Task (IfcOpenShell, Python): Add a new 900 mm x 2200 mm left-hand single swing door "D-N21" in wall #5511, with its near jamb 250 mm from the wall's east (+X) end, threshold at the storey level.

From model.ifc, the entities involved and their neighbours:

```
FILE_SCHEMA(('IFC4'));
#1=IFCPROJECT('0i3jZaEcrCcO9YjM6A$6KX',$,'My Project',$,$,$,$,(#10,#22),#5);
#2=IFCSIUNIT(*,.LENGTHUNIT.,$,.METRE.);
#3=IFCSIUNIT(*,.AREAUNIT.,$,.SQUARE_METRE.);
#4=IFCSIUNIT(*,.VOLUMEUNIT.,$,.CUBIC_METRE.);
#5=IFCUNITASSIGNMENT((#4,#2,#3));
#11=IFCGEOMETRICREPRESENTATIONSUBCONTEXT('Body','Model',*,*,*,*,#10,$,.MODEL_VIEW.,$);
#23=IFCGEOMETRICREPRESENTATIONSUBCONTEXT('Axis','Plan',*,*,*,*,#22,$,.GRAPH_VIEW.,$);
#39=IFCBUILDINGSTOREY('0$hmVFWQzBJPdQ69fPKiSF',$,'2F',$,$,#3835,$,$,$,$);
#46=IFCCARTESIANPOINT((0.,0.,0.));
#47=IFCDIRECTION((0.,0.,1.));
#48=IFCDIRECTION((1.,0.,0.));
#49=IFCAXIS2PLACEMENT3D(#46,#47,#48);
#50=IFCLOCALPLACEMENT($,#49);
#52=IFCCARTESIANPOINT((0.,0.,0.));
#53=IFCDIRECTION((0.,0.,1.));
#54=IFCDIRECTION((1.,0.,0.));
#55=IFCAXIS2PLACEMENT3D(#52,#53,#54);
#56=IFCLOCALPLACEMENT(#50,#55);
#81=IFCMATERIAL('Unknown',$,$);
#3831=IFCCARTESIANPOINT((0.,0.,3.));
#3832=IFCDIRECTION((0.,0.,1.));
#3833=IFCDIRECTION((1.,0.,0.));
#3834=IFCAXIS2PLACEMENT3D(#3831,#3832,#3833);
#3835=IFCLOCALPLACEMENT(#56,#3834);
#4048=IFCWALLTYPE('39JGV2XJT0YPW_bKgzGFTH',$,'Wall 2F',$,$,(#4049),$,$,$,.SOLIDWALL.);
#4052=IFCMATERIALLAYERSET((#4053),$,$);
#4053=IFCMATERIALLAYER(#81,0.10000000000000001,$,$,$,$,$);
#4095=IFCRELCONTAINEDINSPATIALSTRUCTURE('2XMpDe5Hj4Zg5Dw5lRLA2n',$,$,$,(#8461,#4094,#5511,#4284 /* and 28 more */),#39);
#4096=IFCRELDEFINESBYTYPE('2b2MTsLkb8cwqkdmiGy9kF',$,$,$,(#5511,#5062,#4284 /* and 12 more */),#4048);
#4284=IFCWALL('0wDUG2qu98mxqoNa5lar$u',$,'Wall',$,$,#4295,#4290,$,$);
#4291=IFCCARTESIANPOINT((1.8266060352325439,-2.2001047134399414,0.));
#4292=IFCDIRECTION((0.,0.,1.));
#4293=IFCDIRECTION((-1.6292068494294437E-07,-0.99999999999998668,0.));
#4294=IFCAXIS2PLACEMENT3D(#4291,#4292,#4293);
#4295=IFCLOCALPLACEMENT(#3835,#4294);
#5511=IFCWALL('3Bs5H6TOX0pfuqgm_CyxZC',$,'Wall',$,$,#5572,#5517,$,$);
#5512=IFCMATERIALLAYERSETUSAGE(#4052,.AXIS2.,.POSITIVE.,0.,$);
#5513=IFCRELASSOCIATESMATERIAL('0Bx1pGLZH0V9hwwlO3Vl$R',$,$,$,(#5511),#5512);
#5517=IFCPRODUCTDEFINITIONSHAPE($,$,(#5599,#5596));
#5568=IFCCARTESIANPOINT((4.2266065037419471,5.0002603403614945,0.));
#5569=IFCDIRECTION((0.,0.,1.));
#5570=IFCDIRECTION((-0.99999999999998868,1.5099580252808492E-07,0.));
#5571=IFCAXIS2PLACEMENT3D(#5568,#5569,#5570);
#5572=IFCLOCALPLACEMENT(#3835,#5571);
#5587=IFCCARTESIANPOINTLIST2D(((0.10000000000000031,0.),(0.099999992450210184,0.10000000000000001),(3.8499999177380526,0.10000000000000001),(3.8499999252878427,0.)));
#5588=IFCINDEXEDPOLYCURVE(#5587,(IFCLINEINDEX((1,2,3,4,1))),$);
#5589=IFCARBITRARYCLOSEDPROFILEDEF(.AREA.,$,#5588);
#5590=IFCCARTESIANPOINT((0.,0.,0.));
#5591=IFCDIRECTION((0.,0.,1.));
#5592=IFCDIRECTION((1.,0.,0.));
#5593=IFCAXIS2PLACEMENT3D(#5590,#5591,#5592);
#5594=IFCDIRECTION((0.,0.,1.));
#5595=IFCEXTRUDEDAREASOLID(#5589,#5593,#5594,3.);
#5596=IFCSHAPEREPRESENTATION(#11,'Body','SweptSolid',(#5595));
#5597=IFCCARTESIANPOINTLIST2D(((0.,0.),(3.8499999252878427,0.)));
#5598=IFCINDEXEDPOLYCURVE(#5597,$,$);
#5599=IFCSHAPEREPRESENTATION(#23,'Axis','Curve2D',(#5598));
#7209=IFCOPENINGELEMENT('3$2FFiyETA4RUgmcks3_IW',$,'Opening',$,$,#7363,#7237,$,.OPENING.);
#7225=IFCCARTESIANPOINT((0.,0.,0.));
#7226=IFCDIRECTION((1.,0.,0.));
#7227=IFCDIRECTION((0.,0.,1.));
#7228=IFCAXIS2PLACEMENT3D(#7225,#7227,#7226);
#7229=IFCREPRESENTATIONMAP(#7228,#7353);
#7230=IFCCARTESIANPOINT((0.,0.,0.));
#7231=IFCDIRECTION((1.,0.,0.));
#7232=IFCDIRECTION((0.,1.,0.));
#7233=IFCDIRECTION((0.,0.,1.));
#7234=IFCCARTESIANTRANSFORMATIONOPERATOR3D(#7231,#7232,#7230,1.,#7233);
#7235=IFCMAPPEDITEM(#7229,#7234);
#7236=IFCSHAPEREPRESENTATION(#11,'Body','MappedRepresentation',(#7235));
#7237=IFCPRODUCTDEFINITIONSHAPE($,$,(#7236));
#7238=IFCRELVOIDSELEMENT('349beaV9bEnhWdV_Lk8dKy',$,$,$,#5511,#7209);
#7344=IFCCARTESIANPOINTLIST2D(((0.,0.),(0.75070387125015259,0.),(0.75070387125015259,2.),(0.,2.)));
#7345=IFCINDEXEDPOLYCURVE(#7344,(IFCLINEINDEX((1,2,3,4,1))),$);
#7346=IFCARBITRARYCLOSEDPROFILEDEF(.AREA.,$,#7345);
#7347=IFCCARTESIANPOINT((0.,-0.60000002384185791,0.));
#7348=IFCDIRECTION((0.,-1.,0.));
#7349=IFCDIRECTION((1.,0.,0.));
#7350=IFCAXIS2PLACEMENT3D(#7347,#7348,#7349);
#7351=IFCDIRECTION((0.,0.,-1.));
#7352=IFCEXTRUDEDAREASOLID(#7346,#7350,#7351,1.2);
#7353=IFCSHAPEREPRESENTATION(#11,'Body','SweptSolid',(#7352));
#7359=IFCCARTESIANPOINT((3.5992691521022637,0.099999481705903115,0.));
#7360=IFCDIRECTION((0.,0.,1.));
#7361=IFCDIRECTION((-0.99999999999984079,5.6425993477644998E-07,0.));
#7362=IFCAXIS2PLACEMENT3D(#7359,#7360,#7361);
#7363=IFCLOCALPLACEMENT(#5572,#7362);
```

```python
import numpy as np
import ifcopenshell
import ifcopenshell.api.feature
import ifcopenshell.api.geometry
import ifcopenshell.api.root
import ifcopenshell.api.spatial
import ifcopenshell.geom
import ifcopenshell.util.element
import ifcopenshell.util.placement
import ifcopenshell.util.representation
import ifcopenshell.util.shape
import ifcopenshell.util.unit

model = ifcopenshell.open("model.ifc")
unit_scale = ifcopenshell.util.unit.calculate_unit_scale(model)
settings = ifcopenshell.geom.settings()


def volume(element):
    """Net volume in cubic metres, openings subtracted."""
    shape = ifcopenshell.geom.create_shape(settings, element)
    return ifcopenshell.util.shape.get_volume(shape.geometry)


wall = model.by_id(5511)
storey = ifcopenshell.util.element.get_container(wall, ifc_class="IfcBuildingStorey")
context = ifcopenshell.util.representation.get_context(model, "Model", "Body", "MODEL_VIEW")
before = volume(wall)

width, height, from_end, sill = 0.9, 2.2, 0.25, 0.0  # metres

# The wall runs along its own X axis, and the end named is its -X end.
wall_shape = ifcopenshell.geom.create_shape(settings, wall)
x, y, z = ifcopenshell.util.shape.get_vertices(wall_shape.geometry).T
start = x.min() + from_end
face, thickness = float(y.min()), float(y.max() - y.min())
wall_matrix = ifcopenshell.util.placement.get_local_placement(wall.ObjectPlacement)
level = ifcopenshell.util.placement.get_local_placement(storey.ObjectPlacement)[2, 3]


def in_wall(x, y):
    """Placement at x, y metres in the wall's axes, at sill height."""
    matrix = wall_matrix.copy()
    matrix[:, 3] = wall_matrix @ np.array([x / unit_scale, y / unit_scale, 0.0, 1.0])
    matrix[2, 3] = level + sill / unit_scale
    return matrix


# Opening: a box that overshoots both wall faces by 50 mm.
opening = ifcopenshell.api.root.create_entity(model, ifc_class="IfcOpeningElement", predefined_type="OPENING")
box = ifcopenshell.api.geometry.add_wall_representation(
    model, context=context, length=width, height=height, thickness=thickness + 0.1
)
ifcopenshell.api.geometry.assign_representation(model, product=opening, representation=box)
ifcopenshell.api.geometry.edit_object_placement(model, product=opening, matrix=in_wall(start, face - 0.05), is_si=False)
ifcopenshell.api.feature.add_feature(model, feature=opening, element=wall)

door = ifcopenshell.api.root.create_entity(model, ifc_class="IfcDoor", name="D-N21", predefined_type="DOOR")
door.OverallWidth, door.OverallHeight = width / unit_scale, height / unit_scale
door.OperationType = "SINGLE_SWING_LEFT"
body = ifcopenshell.api.geometry.add_door_representation(
    model,
    context=context,
    overall_width=door.OverallWidth,
    overall_height=door.OverallHeight,
    operation_type="SINGLE_SWING_LEFT",
    lining_properties={"LiningDepth": thickness / unit_scale, "ThresholdDepth": thickness / unit_scale},
)
ifcopenshell.api.geometry.assign_representation(model, product=door, representation=body)
ifcopenshell.api.spatial.assign_container(model, products=[door], relating_structure=storey)
ifcopenshell.api.feature.add_filling(model, opening=opening, element=door)

# The lining spans the wall, so the door starts at the wall face.
ifcopenshell.api.geometry.edit_object_placement(model, product=door, matrix=in_wall(start, face), is_si=False)

after = volume(wall)

print(f"wall volume {before:.3f} -> {after:.3f} m3")

model.write("model_v2.ifc")
```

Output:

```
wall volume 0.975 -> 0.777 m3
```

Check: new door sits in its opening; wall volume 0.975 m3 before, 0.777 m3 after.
